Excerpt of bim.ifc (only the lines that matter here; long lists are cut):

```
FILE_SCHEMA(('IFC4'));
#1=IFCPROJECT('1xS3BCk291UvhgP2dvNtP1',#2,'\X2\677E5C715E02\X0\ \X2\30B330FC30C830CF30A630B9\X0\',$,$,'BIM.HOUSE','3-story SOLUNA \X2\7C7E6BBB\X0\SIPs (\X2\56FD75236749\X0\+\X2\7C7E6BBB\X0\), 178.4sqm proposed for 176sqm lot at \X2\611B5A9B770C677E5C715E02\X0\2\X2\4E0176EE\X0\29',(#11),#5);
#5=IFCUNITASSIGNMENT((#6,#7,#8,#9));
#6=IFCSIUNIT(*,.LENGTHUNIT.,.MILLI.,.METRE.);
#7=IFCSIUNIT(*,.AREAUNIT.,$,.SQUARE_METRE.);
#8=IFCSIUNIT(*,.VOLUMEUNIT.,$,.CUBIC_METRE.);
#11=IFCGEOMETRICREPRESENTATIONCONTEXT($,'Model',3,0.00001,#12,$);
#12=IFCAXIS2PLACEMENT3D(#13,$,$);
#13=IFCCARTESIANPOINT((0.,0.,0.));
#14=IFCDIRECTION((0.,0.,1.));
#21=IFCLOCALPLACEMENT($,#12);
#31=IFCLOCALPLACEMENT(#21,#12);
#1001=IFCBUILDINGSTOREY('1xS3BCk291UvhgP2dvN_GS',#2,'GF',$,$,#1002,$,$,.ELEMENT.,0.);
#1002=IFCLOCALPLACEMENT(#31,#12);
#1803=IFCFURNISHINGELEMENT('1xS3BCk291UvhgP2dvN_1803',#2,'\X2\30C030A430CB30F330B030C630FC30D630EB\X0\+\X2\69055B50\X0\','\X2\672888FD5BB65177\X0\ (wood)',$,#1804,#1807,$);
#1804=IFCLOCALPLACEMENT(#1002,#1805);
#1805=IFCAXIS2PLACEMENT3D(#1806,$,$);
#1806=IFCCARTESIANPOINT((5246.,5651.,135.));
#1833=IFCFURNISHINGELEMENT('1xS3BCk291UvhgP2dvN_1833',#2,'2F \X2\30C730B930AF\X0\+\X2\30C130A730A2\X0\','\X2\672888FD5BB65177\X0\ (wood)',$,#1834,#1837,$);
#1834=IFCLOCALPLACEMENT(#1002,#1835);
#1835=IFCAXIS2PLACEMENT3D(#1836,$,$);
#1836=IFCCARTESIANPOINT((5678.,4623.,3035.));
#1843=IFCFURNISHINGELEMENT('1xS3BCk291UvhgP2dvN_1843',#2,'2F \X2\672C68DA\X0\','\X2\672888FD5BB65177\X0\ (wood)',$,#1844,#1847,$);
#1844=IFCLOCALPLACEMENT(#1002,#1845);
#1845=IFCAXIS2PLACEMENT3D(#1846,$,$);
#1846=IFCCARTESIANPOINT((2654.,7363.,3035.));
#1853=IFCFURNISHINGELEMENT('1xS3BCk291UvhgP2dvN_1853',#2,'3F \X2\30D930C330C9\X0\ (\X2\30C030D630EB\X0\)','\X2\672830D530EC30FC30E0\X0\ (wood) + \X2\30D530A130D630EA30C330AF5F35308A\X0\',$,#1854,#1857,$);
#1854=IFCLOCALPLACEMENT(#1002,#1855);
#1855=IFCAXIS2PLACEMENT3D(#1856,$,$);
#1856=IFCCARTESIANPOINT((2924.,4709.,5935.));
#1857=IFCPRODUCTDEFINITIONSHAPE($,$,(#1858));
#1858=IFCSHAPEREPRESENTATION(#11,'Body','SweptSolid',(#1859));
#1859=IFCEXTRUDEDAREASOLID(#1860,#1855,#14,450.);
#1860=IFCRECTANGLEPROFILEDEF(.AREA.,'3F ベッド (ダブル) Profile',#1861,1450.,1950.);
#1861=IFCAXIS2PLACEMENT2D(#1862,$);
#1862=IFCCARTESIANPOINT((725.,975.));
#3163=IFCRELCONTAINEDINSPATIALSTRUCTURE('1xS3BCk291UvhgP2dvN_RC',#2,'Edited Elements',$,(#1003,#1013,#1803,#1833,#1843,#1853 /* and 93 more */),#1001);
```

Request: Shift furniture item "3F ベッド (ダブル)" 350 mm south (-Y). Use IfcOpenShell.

```python
import ifcopenshell
import ifcopenshell.api.geometry
import ifcopenshell.util.placement

model = ifcopenshell.open("bim.ifc")

item = model.by_guid("1xS3BCk291UvhgP2dvN_1853")
matrix = ifcopenshell.util.placement.get_local_placement(item.ObjectPlacement)
matrix[1, 3] -= 350.0
ifcopenshell.api.geometry.edit_object_placement(model, product=item, matrix=matrix, is_si=False)

print(ifcopenshell.util.placement.get_local_placement(item.ObjectPlacement).round(3) + 0.0)

model.write("bim-out.ifc")
```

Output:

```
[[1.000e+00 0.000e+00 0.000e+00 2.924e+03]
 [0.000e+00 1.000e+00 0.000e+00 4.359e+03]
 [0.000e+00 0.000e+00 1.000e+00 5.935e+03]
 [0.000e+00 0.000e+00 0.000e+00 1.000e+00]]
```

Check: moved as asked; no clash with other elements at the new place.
